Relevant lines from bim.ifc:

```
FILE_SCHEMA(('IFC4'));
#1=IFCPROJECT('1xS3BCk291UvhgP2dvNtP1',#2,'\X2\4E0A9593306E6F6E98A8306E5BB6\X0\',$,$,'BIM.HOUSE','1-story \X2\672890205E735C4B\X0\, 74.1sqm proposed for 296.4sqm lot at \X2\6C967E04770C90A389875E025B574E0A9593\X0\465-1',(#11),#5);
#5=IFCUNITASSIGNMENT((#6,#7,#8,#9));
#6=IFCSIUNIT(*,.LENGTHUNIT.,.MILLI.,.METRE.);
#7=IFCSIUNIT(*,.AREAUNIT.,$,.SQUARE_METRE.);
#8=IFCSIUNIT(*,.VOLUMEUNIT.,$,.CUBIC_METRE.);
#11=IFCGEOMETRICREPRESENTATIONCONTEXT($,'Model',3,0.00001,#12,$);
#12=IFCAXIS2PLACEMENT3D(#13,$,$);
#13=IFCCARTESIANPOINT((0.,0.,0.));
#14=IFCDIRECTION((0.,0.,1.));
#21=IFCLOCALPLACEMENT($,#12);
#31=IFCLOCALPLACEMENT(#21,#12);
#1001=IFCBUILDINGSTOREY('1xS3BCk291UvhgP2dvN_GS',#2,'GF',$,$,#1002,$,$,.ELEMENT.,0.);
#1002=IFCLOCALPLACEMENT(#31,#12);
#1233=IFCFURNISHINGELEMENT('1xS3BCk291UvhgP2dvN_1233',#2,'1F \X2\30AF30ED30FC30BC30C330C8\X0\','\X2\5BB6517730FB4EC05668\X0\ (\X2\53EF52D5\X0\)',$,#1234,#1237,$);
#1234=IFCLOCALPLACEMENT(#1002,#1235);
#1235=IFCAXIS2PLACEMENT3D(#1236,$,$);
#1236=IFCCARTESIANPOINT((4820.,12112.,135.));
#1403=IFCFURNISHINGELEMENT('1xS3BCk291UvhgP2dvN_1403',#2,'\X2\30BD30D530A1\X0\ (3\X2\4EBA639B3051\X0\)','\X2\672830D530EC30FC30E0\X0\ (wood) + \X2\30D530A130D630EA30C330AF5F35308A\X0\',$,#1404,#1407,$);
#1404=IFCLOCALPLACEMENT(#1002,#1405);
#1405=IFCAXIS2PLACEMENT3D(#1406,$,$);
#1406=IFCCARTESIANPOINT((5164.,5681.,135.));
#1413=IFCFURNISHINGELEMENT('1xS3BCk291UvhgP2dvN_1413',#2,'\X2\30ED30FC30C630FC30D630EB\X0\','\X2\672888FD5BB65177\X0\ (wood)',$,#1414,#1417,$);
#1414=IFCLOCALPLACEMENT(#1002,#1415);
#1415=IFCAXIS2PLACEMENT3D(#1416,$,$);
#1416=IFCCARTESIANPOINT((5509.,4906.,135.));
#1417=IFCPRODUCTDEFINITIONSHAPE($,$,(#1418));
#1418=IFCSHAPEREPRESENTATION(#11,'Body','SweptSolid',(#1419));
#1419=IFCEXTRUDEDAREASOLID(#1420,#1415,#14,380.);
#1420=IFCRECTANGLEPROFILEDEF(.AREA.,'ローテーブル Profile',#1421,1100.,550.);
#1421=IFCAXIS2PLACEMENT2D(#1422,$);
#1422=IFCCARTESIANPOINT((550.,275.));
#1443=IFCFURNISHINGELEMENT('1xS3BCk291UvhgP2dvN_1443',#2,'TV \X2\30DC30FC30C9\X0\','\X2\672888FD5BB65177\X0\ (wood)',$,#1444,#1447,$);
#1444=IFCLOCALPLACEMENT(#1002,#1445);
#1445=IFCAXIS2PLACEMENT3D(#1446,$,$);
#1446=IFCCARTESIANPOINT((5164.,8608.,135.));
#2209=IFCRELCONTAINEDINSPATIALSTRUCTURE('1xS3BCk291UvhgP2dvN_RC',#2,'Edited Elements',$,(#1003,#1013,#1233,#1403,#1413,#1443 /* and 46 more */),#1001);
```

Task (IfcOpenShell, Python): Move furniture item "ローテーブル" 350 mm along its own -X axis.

```python
import ifcopenshell
import ifcopenshell.api.geometry
import ifcopenshell.util.placement

model = ifcopenshell.open("bim.ifc")

item = model.by_guid("1xS3BCk291UvhgP2dvN_1413")
matrix = ifcopenshell.util.placement.get_local_placement(item.ObjectPlacement)
matrix[:3, 3] -= matrix[:3, 0] * 350.0
ifcopenshell.api.geometry.edit_object_placement(model, product=item, matrix=matrix, is_si=False)

print(ifcopenshell.util.placement.get_local_placement(item.ObjectPlacement).round(3) + 0.0)

model.write("bim_v2.ifc")
```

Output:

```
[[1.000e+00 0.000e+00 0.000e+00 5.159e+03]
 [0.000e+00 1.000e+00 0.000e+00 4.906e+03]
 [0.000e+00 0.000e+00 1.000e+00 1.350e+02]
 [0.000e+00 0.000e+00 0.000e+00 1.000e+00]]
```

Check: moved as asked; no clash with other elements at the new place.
